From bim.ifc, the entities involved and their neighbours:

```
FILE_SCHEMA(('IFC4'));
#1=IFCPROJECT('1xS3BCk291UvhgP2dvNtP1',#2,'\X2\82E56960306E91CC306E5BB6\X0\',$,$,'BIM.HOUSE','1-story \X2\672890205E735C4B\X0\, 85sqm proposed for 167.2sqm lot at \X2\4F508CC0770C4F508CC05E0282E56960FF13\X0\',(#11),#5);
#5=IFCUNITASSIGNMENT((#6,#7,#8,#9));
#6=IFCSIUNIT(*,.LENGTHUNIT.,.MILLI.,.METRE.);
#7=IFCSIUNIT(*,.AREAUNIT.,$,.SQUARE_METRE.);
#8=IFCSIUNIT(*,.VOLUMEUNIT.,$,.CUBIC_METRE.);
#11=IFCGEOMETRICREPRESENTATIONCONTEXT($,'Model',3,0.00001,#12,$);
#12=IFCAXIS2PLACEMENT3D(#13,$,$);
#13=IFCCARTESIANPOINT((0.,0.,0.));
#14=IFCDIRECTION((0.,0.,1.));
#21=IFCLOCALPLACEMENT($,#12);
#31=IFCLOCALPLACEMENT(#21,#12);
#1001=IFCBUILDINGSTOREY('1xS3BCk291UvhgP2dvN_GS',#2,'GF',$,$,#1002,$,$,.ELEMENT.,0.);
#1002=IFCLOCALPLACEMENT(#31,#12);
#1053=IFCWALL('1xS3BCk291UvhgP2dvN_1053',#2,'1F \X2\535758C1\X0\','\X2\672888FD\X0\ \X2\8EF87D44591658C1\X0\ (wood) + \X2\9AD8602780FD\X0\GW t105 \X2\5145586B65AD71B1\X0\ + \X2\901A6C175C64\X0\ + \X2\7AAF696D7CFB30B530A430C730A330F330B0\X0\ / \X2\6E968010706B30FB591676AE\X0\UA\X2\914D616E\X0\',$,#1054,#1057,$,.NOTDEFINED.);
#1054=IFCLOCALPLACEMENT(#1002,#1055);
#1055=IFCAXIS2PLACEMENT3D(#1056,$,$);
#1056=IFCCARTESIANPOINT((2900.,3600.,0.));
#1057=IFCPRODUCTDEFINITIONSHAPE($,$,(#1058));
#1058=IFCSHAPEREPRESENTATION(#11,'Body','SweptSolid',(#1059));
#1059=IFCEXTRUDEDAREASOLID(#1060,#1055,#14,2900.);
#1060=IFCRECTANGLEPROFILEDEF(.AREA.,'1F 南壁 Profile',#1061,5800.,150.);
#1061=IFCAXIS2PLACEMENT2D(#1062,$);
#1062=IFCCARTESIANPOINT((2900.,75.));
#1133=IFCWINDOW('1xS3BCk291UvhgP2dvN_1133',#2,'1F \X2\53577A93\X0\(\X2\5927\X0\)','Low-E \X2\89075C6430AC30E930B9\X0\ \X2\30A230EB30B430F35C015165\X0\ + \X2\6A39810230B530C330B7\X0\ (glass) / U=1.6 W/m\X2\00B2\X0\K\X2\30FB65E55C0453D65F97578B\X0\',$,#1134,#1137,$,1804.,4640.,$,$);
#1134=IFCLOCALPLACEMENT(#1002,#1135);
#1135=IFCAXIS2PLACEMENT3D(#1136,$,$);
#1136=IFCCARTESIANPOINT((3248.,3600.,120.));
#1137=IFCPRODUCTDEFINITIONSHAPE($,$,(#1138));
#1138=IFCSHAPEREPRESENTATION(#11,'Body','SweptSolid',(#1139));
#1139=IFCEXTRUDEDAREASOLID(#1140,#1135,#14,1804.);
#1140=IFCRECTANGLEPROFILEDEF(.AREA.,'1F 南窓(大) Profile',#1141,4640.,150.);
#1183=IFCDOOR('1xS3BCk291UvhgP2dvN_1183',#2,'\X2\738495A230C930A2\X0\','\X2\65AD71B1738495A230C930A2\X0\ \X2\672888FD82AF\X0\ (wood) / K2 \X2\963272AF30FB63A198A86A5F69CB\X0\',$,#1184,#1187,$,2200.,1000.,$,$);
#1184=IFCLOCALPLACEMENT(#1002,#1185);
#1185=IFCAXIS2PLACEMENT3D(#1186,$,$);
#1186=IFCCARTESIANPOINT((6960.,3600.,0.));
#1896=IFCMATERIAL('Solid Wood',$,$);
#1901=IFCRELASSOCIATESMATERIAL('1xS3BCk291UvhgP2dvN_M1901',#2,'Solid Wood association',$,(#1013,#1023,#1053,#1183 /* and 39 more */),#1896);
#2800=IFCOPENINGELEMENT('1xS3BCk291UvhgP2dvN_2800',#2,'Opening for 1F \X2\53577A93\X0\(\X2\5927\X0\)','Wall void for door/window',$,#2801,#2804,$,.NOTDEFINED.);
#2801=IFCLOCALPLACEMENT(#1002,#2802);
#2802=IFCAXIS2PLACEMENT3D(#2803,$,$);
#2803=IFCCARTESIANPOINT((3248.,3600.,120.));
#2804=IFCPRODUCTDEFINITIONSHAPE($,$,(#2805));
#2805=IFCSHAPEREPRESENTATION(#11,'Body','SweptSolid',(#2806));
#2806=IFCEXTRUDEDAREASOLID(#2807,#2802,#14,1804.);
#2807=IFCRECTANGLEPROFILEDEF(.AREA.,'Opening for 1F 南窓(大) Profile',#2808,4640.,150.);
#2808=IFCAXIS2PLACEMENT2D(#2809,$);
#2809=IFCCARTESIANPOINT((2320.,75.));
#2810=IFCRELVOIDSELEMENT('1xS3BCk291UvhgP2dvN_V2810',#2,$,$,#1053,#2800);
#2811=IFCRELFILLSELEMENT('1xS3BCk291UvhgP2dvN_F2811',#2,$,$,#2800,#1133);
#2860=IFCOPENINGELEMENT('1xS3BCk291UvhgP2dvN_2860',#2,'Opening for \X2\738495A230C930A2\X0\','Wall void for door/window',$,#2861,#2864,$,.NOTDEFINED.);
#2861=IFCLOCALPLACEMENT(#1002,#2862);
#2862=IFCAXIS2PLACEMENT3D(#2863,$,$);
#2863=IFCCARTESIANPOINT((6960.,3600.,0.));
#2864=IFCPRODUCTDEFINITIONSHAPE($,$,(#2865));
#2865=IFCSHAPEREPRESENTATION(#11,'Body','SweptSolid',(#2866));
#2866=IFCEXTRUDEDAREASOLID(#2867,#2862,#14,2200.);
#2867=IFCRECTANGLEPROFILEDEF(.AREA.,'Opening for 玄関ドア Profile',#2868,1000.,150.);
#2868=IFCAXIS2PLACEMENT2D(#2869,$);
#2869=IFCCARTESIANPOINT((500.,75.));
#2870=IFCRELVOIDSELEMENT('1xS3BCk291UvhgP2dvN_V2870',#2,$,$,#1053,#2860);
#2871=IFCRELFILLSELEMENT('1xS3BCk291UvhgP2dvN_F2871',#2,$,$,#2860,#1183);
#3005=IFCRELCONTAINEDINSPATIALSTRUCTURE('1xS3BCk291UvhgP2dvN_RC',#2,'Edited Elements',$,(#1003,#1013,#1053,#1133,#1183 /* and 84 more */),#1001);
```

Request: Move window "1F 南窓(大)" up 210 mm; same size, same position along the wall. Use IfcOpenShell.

```python
import numpy as np
import ifcopenshell
import ifcopenshell.api.geometry
import ifcopenshell.util.placement
import ifcopenshell.util.unit

model = ifcopenshell.open("bim.ifc")
unit_scale = ifcopenshell.util.unit.calculate_unit_scale(model)

window = model.by_id(1133)
opening = window.FillsVoids[0].RelatingOpeningElement
dz = 0.21 / unit_scale

shift = np.array([0.0, 0.0, dz])
# The window is not placed relative to its opening, so move both.
for product in (opening, window):
    matrix = ifcopenshell.util.placement.get_local_placement(product.ObjectPlacement)
    matrix[:3, 3] += shift
    ifcopenshell.api.geometry.edit_object_placement(model, product=product, matrix=matrix, is_si=False)

print(f"moved by {dz * unit_scale:+.3f} m")

model.write("bim_rev.ifc")
```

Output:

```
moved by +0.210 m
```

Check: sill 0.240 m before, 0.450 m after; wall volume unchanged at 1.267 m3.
